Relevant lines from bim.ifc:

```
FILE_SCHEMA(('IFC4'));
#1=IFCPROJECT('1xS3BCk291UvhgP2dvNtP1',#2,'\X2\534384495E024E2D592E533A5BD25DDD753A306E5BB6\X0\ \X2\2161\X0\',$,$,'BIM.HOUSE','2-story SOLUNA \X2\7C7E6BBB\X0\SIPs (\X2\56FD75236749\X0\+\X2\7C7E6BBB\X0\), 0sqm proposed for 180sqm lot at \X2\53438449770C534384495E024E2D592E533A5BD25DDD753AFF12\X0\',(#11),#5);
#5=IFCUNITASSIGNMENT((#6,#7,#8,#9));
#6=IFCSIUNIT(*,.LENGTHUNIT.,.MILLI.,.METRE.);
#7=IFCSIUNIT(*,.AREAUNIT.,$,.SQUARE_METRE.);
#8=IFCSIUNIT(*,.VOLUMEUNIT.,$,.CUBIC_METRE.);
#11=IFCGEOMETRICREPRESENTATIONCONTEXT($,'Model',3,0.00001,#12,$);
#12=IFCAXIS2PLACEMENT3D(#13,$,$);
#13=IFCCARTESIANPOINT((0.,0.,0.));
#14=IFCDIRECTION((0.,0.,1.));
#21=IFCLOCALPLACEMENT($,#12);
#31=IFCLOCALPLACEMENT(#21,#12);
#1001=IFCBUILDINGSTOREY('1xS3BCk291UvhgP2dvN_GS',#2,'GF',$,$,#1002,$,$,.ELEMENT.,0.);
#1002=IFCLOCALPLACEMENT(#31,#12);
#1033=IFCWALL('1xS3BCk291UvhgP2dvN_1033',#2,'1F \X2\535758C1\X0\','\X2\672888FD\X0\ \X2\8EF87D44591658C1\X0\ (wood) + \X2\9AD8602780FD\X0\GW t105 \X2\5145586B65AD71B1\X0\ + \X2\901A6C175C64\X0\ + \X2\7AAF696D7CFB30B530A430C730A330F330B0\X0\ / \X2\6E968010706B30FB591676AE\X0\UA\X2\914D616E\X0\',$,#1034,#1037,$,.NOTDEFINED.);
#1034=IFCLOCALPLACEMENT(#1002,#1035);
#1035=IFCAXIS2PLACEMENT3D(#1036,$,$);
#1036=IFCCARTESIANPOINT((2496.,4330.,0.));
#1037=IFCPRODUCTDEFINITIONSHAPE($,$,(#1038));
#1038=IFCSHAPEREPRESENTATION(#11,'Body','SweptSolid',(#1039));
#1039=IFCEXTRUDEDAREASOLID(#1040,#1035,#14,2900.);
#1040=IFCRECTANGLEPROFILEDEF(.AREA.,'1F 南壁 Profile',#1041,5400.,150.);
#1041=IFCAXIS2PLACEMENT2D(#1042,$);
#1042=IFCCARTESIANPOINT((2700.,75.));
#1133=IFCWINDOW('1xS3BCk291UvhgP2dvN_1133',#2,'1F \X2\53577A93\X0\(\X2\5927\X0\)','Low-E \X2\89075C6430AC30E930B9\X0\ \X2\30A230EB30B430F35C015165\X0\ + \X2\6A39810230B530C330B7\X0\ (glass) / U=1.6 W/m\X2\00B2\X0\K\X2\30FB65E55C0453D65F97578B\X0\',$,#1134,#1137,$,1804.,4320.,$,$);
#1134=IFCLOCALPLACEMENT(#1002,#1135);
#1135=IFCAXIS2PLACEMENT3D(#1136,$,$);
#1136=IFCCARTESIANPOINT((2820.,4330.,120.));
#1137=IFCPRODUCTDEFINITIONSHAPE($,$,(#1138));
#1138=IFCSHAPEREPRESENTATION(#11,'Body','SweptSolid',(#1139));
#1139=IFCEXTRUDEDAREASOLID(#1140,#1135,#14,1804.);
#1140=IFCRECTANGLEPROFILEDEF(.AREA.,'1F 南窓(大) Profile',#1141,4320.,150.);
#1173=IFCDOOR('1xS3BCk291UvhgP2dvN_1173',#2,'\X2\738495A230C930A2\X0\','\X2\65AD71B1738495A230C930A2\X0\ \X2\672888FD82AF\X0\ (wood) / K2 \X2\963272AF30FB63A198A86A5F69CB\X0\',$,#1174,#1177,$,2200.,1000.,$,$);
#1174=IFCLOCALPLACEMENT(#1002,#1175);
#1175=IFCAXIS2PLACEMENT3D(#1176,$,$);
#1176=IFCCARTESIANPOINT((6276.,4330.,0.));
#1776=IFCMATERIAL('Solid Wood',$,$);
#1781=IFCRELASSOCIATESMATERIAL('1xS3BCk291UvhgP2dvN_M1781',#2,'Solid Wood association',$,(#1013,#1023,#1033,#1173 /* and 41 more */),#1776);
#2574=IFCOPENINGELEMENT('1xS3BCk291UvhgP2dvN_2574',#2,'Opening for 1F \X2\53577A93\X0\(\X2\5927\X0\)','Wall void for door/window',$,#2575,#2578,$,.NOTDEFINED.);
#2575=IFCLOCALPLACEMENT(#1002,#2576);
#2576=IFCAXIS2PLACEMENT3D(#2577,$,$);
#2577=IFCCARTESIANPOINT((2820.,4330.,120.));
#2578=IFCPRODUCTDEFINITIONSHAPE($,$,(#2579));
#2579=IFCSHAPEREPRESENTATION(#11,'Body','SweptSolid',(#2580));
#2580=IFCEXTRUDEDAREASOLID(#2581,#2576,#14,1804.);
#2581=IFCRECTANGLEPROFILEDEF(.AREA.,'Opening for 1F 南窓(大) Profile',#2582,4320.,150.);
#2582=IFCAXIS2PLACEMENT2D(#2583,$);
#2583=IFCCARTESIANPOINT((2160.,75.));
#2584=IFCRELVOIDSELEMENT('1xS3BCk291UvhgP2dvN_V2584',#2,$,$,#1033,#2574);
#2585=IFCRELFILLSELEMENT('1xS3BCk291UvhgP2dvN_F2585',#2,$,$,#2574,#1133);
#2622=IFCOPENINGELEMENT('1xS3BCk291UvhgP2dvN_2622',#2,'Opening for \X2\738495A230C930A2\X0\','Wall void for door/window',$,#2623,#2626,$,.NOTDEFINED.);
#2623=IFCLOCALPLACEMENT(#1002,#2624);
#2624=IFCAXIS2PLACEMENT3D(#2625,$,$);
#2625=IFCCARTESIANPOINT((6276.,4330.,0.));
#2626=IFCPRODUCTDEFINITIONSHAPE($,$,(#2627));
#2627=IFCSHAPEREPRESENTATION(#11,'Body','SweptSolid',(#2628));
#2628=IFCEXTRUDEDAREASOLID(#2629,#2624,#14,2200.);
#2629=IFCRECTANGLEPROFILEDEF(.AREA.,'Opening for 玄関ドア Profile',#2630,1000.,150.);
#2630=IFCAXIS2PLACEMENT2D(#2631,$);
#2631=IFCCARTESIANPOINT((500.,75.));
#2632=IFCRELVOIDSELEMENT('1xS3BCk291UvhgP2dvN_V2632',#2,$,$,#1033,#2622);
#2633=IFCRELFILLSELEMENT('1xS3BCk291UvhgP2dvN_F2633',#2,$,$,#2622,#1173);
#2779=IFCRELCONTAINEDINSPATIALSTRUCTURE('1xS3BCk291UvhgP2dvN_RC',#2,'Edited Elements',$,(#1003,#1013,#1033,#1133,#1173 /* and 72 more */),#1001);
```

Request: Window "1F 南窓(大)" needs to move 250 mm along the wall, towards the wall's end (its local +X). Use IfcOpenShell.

```python
import ifcopenshell
import ifcopenshell.api.geometry
import ifcopenshell.util.placement

model = ifcopenshell.open("bim.ifc")

window = model.by_id(1133)
opening = window.FillsVoids[0].RelatingOpeningElement
wall = opening.VoidsElements[0].RelatingBuildingElement

wall_matrix = ifcopenshell.util.placement.get_local_placement(wall.ObjectPlacement)
shift = wall_matrix[:3, 0] * 250.0
before = ifcopenshell.util.placement.get_local_placement(window.ObjectPlacement)[:3, 3].copy()

# The window is not placed relative to its opening, so move both.
for product in (opening, window):
    matrix = ifcopenshell.util.placement.get_local_placement(product.ObjectPlacement)
    matrix[:3, 3] += shift
    ifcopenshell.api.geometry.edit_object_placement(model, product=product, matrix=matrix, is_si=False)

after = ifcopenshell.util.placement.get_local_placement(window.ObjectPlacement)[:3, 3]
print("window moved by", (after - before).round(3) + 0.0)

model.write("bim_edited.ifc")
```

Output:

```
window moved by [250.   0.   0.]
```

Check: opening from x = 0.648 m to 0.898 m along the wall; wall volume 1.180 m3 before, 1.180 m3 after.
